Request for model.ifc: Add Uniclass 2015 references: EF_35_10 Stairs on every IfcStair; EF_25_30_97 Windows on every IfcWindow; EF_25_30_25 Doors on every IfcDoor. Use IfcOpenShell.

First a look at what the model holds.

```python
import ifcopenshell

model = ifcopenshell.open("model.ifc")
print(model.schema)
print("classifications:", [c.Name for c in model.by_type("IfcClassification")])
for ifc_class in ("IfcDoor", "IfcRoof", "IfcStair", "IfcWall", "IfcWindow"):
    print(ifc_class, len(model.by_type(ifc_class)))
```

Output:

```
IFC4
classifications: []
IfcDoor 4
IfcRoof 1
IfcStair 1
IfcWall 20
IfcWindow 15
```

```python
import ifcopenshell
import ifcopenshell.api.classification

model = ifcopenshell.open("model.ifc")

system = ifcopenshell.api.classification.add_classification(model, classification="Uniclass 2015")

codes = {
    "IfcStair": ("EF_35_10", "Stairs"),
    "IfcWindow": ("EF_25_30_97", "Windows"),
    "IfcDoor": ("EF_25_30_25", "Doors"),
}
for ifc_class, (code, name) in codes.items():
    products = model.by_type(ifc_class)
    ifcopenshell.api.classification.add_reference(
        model, products=products, classification=system, identification=code, name=name
    )
    print(code, len(products))

model.write("model-out.ifc")
```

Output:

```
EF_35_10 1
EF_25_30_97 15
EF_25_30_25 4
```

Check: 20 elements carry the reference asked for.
